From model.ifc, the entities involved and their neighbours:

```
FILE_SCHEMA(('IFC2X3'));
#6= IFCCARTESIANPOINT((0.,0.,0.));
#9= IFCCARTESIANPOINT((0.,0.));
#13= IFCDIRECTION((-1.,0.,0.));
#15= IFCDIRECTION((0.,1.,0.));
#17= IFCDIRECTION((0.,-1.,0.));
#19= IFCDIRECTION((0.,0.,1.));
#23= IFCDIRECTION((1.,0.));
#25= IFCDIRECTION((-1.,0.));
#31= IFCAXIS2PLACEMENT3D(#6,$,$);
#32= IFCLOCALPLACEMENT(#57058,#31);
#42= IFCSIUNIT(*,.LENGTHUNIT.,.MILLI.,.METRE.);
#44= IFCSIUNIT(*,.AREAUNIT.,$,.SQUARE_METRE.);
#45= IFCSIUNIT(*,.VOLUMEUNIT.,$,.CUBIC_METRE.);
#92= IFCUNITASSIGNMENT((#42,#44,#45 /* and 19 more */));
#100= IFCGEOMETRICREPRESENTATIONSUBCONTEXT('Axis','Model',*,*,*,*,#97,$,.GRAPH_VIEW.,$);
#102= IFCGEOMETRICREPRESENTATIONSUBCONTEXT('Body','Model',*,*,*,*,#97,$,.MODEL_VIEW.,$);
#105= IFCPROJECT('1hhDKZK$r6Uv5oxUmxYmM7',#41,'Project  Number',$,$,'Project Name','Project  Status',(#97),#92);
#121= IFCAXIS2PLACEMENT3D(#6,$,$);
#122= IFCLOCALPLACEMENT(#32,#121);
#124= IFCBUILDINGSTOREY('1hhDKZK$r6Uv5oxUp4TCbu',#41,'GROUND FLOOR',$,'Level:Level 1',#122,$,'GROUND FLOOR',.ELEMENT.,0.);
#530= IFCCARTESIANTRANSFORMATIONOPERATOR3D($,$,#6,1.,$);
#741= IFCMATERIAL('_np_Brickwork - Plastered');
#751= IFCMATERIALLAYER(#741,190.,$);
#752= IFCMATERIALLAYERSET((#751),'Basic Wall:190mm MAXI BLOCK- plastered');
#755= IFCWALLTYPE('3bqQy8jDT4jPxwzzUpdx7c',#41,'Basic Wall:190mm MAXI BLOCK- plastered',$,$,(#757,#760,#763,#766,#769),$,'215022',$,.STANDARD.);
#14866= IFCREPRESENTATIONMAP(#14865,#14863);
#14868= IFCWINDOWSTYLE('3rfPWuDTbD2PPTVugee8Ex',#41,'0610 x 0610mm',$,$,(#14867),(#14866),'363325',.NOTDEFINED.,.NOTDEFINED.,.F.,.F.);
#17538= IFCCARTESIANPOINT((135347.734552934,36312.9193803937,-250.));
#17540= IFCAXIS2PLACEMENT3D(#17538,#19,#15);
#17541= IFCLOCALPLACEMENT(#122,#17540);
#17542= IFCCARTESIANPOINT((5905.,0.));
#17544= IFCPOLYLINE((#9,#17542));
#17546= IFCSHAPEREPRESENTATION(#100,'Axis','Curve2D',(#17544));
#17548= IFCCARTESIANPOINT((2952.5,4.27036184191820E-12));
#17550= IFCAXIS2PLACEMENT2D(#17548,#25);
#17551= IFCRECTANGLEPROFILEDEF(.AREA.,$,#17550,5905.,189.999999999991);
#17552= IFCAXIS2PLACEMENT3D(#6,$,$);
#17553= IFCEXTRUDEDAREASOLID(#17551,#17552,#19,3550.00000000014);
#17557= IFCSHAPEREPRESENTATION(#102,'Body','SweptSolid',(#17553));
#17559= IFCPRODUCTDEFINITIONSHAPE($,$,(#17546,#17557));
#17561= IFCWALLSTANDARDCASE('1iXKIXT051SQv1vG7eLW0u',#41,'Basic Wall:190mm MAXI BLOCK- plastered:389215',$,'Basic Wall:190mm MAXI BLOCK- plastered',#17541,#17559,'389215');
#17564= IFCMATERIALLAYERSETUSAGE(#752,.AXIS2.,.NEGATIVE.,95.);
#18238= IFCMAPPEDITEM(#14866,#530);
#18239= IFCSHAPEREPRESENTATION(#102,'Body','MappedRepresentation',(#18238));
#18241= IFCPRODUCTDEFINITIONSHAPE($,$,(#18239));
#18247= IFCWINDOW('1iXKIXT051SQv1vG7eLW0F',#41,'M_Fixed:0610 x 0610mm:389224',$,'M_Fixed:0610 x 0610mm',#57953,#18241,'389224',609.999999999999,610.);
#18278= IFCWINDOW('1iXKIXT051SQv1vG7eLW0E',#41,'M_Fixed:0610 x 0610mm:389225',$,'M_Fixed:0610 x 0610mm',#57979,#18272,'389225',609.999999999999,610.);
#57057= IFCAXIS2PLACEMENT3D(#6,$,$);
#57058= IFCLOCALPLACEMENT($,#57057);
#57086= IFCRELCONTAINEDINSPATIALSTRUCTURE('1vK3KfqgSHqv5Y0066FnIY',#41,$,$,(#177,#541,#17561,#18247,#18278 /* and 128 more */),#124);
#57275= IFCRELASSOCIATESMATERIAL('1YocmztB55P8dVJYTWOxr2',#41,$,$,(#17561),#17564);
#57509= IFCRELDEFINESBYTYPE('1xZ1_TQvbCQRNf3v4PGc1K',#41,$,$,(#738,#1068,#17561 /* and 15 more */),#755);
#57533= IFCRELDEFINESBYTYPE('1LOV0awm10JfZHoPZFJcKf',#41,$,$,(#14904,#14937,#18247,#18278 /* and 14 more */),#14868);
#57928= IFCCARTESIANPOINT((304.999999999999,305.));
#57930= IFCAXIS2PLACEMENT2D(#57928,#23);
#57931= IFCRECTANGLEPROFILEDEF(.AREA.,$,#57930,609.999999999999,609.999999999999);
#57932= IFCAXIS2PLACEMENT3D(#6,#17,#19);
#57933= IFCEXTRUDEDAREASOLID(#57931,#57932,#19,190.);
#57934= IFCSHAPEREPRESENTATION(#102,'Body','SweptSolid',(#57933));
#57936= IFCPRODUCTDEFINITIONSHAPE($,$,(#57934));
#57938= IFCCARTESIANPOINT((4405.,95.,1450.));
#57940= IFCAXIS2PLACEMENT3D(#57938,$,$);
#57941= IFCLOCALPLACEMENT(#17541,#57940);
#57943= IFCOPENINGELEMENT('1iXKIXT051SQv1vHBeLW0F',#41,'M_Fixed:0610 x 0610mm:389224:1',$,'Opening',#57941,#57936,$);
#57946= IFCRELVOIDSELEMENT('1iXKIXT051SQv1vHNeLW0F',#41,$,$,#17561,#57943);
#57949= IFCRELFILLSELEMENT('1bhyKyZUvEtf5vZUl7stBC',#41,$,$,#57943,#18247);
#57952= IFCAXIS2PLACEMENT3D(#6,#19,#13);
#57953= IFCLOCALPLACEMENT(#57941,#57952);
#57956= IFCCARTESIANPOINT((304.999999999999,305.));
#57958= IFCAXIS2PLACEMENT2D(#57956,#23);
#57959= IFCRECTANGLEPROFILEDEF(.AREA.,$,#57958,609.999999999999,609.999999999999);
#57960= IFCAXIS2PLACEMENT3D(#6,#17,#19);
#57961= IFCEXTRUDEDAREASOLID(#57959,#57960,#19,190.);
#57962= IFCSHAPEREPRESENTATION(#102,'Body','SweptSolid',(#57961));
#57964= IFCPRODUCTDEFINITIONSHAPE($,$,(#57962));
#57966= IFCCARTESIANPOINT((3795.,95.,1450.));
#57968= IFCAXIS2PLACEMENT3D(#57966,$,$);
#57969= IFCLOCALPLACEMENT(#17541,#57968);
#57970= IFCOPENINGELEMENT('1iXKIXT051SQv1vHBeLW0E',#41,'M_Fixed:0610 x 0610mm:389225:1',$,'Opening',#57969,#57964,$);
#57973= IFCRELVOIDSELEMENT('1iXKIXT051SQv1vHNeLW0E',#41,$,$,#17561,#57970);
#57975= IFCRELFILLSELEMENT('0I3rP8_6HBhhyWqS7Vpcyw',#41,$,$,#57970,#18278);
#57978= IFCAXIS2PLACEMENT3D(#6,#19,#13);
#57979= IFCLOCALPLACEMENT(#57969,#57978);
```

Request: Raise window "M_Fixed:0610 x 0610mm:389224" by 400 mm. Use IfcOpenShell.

```python
import numpy as np
import ifcopenshell
import ifcopenshell.api.geometry
import ifcopenshell.util.placement
import ifcopenshell.util.unit

model = ifcopenshell.open("model.ifc")
unit_scale = ifcopenshell.util.unit.calculate_unit_scale(model)

window = model.by_guid("1iXKIXT051SQv1vG7eLW0F")
opening = window.FillsVoids[0].RelatingOpeningElement
dz = 400.0

shift = np.array([0.0, 0.0, dz])
# The window is placed relative to its opening, so it follows when the opening moves.
matrix = ifcopenshell.util.placement.get_local_placement(opening.ObjectPlacement)
matrix[:3, 3] += shift
ifcopenshell.api.geometry.edit_object_placement(
    model, product=opening, matrix=matrix, is_si=False, should_transform_children=True
)

print(f"moved by {dz * unit_scale:+.3f} m")

model.write("model-out.ifc")
```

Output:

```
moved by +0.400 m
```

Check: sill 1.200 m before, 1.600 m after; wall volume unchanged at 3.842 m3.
